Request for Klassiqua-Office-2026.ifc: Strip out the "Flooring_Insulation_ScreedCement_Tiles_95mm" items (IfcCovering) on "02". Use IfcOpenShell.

First a look at what the model holds.

```python
import ifcopenshell
import ifcopenshell.util.element

model = ifcopenshell.open("Klassiqua-Office-2026.ifc")
print(model.schema)
storey = next(s for s in model.by_type("IfcBuildingStorey") if s.Name == "02")
coverings = [e for e in ifcopenshell.util.element.get_decomposition(storey) if e.is_a("IfcCovering")]
seen = {}
for e in coverings:
    element_type = ifcopenshell.util.element.get_type(e)
    name = element_type.Name if element_type not in (None, e) else None
    seen[name] = seen.get(name, 0) + 1
for name, count in sorted(seen.items(), key=str):
    print(count, "x", name)
```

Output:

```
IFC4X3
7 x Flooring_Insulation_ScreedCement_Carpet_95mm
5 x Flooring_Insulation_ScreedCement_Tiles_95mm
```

```python
import ifcopenshell
import ifcopenshell.api.root
import ifcopenshell.util.element

model = ifcopenshell.open("Klassiqua-Office-2026.ifc")

storey = next(s for s in model.by_type("IfcBuildingStorey") if s.Name == "02")
coverings = [e for e in ifcopenshell.util.element.get_decomposition(storey) if e.is_a("IfcCovering")]
targets = [e for e in coverings if (t := ifcopenshell.util.element.get_type(e)) not in (None, e) and t.Name == "Flooring_Insulation_ScreedCement_Tiles_95mm"]

for e in targets:
    ifcopenshell.api.root.remove_product(model, product=e)
print(len(targets), "removed")

model.write("Klassiqua-Office-2026_edited.ifc")
```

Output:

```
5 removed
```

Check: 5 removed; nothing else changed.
